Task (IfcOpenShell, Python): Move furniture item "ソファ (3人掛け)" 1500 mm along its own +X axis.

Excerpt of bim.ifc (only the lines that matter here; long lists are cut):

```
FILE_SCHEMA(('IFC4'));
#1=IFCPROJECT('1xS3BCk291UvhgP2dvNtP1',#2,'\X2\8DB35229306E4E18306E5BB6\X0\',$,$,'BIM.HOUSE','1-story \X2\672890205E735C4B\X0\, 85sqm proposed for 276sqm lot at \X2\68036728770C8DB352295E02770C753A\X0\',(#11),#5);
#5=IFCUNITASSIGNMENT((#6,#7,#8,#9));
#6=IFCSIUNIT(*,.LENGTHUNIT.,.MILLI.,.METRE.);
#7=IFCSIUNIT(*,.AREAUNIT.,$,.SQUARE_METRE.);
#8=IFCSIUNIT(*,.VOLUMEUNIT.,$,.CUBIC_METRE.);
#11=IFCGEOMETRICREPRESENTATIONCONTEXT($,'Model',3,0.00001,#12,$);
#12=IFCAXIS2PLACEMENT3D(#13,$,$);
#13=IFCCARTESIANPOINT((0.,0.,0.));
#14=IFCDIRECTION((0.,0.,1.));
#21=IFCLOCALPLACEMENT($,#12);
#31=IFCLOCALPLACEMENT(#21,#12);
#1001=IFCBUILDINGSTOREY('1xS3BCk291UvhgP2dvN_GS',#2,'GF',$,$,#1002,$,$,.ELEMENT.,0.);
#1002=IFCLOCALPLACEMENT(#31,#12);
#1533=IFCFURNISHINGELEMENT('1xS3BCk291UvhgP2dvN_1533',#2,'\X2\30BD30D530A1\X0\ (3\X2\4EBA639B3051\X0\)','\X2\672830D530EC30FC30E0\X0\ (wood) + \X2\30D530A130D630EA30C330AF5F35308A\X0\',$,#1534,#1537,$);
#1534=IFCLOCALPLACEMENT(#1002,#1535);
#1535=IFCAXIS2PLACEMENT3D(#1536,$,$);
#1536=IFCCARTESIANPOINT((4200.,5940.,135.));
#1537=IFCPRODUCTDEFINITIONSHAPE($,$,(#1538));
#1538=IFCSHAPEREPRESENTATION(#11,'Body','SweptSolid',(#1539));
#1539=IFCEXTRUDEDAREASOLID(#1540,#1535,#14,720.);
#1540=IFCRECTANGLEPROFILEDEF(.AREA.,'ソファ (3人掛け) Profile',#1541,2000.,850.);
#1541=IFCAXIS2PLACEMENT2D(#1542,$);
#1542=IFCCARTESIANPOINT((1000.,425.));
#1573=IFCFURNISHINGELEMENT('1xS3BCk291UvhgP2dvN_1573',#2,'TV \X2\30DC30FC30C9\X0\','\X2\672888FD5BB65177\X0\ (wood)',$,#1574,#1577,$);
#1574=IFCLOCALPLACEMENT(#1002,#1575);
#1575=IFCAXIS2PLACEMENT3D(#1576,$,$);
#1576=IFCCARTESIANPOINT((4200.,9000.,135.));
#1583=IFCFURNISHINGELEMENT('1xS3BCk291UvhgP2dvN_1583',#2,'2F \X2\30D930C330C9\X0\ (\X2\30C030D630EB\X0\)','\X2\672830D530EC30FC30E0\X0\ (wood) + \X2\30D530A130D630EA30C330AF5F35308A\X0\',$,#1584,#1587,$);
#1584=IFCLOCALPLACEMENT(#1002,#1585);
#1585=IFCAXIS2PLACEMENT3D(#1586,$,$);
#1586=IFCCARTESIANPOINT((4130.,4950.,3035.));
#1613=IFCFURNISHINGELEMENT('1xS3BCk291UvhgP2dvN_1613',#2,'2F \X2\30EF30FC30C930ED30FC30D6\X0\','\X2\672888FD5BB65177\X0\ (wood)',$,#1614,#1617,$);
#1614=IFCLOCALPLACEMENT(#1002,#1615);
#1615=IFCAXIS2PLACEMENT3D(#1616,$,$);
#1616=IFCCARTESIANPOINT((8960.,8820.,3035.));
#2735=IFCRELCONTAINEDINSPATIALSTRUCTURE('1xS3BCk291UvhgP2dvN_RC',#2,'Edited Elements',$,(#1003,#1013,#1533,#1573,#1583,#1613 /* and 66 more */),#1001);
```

```python
import ifcopenshell
import ifcopenshell.api.geometry
import ifcopenshell.util.placement

model = ifcopenshell.open("bim.ifc")

item = model.by_id(1533)
matrix = ifcopenshell.util.placement.get_local_placement(item.ObjectPlacement)
matrix[:3, 3] += matrix[:3, 0] * 1500.0
ifcopenshell.api.geometry.edit_object_placement(model, product=item, matrix=matrix, is_si=False)

print(ifcopenshell.util.placement.get_local_placement(item.ObjectPlacement).round(3) + 0.0)

model.write("bim-out.ifc")
```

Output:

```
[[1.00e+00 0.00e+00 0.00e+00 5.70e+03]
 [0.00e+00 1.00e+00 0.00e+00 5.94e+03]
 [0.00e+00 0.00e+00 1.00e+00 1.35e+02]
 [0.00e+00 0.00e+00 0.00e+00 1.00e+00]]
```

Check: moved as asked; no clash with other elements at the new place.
